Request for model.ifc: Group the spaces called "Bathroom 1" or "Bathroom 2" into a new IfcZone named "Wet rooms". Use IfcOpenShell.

First a look at what the model holds.

```python
import ifcopenshell

model = ifcopenshell.open("model.ifc")
print(model.schema)
seen = {}
for space in model.by_type("IfcSpace"):
    seen[space.LongName] = seen.get(space.LongName, 0) + 1
for name, count in sorted(seen.items(), key=str):
    print(count, "x", name)
print("zones:", [z.Name for z in model.by_type("IfcZone")][:20])
```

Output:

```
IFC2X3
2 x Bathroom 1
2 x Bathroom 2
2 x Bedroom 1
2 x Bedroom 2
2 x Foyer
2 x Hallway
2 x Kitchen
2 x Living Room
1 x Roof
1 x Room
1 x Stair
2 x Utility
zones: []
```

```python
import ifcopenshell
import ifcopenshell.api.group
import ifcopenshell.api.root

model = ifcopenshell.open("model.ifc")

names = {"Bathroom 1", "Bathroom 2"}
spaces = [s for s in model.by_type("IfcSpace") if s.LongName in names]

zone = ifcopenshell.api.root.create_entity(model, ifc_class="IfcZone", name="Wet rooms")
ifcopenshell.api.group.assign_group(model, products=spaces, group=zone)
print(len(spaces), "spaces in", zone.Name)

model.write("model-out.ifc")
```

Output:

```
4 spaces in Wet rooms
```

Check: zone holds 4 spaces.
